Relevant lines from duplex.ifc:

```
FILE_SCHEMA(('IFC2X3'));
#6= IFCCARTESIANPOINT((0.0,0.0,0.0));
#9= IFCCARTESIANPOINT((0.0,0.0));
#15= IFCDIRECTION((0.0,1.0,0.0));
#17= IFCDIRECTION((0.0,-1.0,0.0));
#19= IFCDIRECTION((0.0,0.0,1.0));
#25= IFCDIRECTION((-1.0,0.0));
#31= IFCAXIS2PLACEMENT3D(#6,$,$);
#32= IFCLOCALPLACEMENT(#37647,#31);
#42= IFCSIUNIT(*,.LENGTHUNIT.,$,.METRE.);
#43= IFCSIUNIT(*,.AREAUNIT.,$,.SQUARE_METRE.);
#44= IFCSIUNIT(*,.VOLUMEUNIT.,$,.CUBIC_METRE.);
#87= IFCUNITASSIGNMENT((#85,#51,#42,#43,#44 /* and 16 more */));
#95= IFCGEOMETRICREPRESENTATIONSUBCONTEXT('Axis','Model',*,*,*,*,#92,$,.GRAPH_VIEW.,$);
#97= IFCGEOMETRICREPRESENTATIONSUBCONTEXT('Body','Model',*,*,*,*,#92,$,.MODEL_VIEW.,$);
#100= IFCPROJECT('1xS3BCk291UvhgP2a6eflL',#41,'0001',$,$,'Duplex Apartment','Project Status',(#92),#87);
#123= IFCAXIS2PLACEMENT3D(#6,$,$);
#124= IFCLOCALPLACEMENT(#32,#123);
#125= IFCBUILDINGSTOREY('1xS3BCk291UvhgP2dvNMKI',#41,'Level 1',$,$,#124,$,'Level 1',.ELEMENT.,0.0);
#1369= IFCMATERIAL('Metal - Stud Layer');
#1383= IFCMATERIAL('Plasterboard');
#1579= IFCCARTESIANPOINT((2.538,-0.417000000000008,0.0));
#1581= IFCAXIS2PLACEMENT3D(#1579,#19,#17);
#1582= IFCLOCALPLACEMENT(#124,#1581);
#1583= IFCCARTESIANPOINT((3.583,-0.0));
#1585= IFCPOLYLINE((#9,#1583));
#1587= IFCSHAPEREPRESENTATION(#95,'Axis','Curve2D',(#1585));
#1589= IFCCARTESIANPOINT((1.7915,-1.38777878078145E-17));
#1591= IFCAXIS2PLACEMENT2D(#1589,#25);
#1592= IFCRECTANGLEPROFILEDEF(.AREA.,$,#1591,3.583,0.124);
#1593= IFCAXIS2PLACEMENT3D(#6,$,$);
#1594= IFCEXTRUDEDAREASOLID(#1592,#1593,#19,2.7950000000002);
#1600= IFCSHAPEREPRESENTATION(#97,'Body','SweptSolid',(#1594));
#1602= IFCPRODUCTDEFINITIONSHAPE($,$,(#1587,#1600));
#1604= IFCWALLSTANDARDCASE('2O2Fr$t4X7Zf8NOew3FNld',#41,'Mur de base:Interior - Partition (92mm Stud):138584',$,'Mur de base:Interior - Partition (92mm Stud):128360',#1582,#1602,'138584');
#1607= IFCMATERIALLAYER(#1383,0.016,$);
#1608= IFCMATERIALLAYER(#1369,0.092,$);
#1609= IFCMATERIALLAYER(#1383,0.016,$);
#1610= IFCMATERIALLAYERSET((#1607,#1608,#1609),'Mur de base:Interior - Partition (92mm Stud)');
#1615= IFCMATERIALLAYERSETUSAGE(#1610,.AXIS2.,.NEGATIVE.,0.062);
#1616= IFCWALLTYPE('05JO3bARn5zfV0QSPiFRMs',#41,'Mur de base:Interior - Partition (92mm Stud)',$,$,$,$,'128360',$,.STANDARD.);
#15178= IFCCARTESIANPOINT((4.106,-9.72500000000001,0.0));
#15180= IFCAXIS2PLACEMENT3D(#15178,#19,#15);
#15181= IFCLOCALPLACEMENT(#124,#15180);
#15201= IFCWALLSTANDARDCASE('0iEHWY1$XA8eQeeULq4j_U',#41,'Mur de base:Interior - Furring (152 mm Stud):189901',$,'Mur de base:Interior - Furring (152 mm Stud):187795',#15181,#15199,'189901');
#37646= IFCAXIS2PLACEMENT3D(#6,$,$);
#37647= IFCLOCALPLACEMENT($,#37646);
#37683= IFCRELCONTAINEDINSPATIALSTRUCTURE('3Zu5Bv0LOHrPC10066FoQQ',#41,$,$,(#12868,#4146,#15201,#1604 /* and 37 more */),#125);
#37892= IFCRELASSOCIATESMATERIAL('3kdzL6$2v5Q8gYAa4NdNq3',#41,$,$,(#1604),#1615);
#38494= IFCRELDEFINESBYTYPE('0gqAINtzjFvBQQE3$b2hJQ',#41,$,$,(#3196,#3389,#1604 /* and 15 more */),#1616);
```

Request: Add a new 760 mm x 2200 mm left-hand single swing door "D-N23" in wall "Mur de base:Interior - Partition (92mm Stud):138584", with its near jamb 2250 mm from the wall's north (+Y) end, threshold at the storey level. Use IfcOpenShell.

```python
import numpy as np
import ifcopenshell
import ifcopenshell.api.feature
import ifcopenshell.api.geometry
import ifcopenshell.api.root
import ifcopenshell.api.spatial
import ifcopenshell.api.type
import ifcopenshell.geom
import ifcopenshell.util.element
import ifcopenshell.util.placement
import ifcopenshell.util.representation
import ifcopenshell.util.shape
import ifcopenshell.util.unit

model = ifcopenshell.open("duplex.ifc")
unit_scale = ifcopenshell.util.unit.calculate_unit_scale(model)
settings = ifcopenshell.geom.settings()


def volume(element):
    """Net volume in cubic metres, openings subtracted."""
    shape = ifcopenshell.geom.create_shape(settings, element)
    return ifcopenshell.util.shape.get_volume(shape.geometry)


wall = model.by_guid("2O2Fr$t4X7Zf8NOew3FNld")
storey = ifcopenshell.util.element.get_container(wall, ifc_class="IfcBuildingStorey")
context = ifcopenshell.util.representation.get_context(model, "Model", "Body", "MODEL_VIEW")
before = volume(wall)

width, height, from_end, sill = 0.76, 2.2, 2.25, 0.0  # metres

# The wall runs along its own X axis, and the end named is its -X end.
wall_shape = ifcopenshell.geom.create_shape(settings, wall)
x, y, z = ifcopenshell.util.shape.get_vertices(wall_shape.geometry).T
start = x.min() + from_end
face, thickness = float(y.min()), float(y.max() - y.min())
wall_matrix = ifcopenshell.util.placement.get_local_placement(wall.ObjectPlacement)
level = ifcopenshell.util.placement.get_local_placement(storey.ObjectPlacement)[2, 3]


def in_wall(x, y):
    """Placement at x, y metres in the wall's axes, at sill height."""
    matrix = wall_matrix.copy()
    matrix[:, 3] = wall_matrix @ np.array([x / unit_scale, y / unit_scale, 0.0, 1.0])
    matrix[2, 3] = level + sill / unit_scale
    return matrix


# Opening: a box that overshoots both wall faces by 50 mm.
opening = ifcopenshell.api.root.create_entity(model, ifc_class="IfcOpeningElement")
box = ifcopenshell.api.geometry.add_wall_representation(
    model, context=context, length=width, height=height, thickness=thickness + 0.1
)
ifcopenshell.api.geometry.assign_representation(model, product=opening, representation=box)
ifcopenshell.api.geometry.edit_object_placement(model, product=opening, matrix=in_wall(start, face - 0.05), is_si=False)
ifcopenshell.api.feature.add_feature(model, feature=opening, element=wall)

door = ifcopenshell.api.root.create_entity(model, ifc_class="IfcDoor", name="D-N23")
door.OverallWidth, door.OverallHeight = width / unit_scale, height / unit_scale
body = ifcopenshell.api.geometry.add_door_representation(
    model,
    context=context,
    overall_width=door.OverallWidth,
    overall_height=door.OverallHeight,
    operation_type="SINGLE_SWING_LEFT",
    lining_properties={"LiningDepth": thickness / unit_scale, "ThresholdDepth": thickness / unit_scale},
)
ifcopenshell.api.geometry.assign_representation(model, product=door, representation=body)
ifcopenshell.api.spatial.assign_container(model, products=[door], relating_structure=storey)
fills = ifcopenshell.api.feature.add_filling(model, opening=opening, element=door)
fills.OwnerHistory = door.OwnerHistory  # required in IFC2X3

# IFC2X3 keeps the operation on the door style.
style = ifcopenshell.api.root.create_entity(model, ifc_class="IfcDoorStyle", name="D-N23")
style.OperationType, style.ConstructionType = "SINGLE_SWING_LEFT", "NOTDEFINED"
style.ParameterTakesPrecedence = style.Sizeable = False
ifcopenshell.api.type.assign_type(model, related_objects=[door], relating_type=style)

# The lining spans the wall, so the door starts at the wall face.
ifcopenshell.api.geometry.edit_object_placement(model, product=door, matrix=in_wall(start, face), is_si=False)

after = volume(wall)

print(f"wall volume {before:.3f} -> {after:.3f} m3")

model.write("duplex-out.ifc")
```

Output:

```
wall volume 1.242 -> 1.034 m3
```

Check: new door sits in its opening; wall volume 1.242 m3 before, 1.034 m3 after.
